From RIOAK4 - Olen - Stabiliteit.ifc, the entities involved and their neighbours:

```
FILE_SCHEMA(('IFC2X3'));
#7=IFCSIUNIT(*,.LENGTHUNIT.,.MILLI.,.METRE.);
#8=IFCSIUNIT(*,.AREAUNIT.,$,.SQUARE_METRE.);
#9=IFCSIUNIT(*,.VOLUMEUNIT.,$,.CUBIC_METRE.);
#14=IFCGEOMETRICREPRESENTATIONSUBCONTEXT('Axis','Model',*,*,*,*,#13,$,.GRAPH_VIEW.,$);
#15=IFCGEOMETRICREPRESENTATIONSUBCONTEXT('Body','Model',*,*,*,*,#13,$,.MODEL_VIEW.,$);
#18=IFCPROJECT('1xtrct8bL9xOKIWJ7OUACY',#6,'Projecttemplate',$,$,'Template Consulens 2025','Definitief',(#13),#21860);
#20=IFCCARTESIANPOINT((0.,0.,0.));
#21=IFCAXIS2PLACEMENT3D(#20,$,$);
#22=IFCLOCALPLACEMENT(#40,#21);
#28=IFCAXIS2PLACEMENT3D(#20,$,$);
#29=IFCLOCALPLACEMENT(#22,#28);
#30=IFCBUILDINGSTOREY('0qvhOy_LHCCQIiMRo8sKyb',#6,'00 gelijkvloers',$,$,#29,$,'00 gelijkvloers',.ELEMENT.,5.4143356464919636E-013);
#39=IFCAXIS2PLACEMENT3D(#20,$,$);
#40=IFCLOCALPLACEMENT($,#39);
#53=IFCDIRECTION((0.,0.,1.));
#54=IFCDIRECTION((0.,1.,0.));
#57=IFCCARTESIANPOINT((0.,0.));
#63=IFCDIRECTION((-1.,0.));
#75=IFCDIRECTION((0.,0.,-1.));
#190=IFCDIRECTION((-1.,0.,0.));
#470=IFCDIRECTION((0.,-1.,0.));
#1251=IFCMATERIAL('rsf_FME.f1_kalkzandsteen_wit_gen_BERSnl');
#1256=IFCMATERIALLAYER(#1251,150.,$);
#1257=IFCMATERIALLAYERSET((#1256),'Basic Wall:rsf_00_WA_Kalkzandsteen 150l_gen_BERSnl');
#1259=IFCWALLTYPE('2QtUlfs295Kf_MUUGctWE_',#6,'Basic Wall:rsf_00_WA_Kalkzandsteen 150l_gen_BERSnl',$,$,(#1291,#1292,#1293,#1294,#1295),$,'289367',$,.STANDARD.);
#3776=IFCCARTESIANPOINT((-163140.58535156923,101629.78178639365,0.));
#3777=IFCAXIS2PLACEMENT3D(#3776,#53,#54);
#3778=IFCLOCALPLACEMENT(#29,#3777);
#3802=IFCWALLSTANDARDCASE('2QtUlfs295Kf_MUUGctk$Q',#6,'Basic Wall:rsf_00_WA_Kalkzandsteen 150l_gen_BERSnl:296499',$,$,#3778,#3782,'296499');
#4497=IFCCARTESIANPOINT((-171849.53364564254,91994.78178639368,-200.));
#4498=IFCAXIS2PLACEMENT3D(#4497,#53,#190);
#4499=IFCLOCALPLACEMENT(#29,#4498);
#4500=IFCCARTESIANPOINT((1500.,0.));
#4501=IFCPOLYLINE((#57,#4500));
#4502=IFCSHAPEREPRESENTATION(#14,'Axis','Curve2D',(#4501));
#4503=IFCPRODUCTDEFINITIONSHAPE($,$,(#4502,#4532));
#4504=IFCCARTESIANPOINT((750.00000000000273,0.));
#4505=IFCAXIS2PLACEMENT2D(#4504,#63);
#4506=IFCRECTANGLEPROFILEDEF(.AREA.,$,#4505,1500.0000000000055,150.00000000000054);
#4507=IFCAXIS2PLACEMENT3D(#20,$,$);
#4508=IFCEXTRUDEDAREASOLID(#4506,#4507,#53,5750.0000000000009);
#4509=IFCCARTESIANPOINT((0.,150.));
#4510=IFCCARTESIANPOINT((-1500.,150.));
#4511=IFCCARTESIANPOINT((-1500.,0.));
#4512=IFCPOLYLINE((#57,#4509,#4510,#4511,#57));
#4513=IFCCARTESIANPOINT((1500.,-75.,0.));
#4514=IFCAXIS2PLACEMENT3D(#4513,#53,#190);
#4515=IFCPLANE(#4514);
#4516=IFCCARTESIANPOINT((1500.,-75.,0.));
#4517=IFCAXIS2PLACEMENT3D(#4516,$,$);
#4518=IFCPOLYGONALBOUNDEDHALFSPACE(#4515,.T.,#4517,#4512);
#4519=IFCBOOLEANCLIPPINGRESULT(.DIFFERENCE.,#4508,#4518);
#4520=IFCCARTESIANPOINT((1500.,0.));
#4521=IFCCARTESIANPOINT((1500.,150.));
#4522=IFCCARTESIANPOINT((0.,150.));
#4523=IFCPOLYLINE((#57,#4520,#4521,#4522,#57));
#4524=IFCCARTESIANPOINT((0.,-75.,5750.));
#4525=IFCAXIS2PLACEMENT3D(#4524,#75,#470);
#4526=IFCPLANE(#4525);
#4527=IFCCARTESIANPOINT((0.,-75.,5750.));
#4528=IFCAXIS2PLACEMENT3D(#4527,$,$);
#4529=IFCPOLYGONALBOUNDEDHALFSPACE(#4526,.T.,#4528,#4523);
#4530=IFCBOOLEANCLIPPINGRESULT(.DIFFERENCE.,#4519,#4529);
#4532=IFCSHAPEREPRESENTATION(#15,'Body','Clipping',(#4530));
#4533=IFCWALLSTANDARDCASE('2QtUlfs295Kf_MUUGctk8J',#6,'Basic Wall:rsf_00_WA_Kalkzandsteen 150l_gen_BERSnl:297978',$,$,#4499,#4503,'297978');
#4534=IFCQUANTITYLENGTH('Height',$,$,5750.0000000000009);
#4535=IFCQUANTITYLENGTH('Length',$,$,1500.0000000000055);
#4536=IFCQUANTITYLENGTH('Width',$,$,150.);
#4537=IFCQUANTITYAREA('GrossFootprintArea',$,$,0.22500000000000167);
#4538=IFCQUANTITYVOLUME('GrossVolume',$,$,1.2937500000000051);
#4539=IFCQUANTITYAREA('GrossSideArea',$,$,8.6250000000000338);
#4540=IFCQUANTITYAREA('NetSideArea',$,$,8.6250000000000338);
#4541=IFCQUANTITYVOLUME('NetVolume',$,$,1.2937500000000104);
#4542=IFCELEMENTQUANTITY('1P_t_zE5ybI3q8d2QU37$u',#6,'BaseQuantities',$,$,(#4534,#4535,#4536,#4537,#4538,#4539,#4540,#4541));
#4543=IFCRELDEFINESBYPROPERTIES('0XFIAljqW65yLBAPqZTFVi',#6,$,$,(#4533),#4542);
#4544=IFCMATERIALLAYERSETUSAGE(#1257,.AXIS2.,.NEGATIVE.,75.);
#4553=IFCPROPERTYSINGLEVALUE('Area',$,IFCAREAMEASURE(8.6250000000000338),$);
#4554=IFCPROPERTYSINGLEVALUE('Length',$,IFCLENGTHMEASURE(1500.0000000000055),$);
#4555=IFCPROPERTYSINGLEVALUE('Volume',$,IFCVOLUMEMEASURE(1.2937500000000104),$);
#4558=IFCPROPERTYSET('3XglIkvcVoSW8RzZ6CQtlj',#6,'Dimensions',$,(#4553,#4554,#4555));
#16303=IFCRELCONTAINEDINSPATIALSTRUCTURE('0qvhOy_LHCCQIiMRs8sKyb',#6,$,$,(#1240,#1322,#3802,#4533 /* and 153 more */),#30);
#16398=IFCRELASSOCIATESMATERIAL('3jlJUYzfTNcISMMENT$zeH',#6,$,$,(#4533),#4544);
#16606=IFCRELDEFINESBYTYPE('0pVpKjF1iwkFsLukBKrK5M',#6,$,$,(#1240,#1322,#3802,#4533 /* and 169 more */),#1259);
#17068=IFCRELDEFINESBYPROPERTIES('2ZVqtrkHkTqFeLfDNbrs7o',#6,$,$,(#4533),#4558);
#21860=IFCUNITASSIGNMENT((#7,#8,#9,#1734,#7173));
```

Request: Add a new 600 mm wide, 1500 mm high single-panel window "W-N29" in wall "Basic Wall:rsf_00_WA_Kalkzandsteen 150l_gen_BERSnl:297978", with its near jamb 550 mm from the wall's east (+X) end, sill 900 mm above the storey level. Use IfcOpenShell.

```python
import numpy as np
import ifcopenshell
import ifcopenshell.api.feature
import ifcopenshell.api.geometry
import ifcopenshell.api.pset
import ifcopenshell.api.root
import ifcopenshell.api.spatial
import ifcopenshell.api.type
import ifcopenshell.geom
import ifcopenshell.util.element
import ifcopenshell.util.placement
import ifcopenshell.util.representation
import ifcopenshell.util.shape
import ifcopenshell.util.unit

model = ifcopenshell.open("RIOAK4 - Olen - Stabiliteit.ifc")
unit_scale = ifcopenshell.util.unit.calculate_unit_scale(model)
area_scale = ifcopenshell.util.unit.calculate_unit_scale(model, "AREAUNIT")
volume_scale = ifcopenshell.util.unit.calculate_unit_scale(model, "VOLUMEUNIT")
settings = ifcopenshell.geom.settings()


def volume(element):
    """Net volume in cubic metres, openings subtracted."""
    shape = ifcopenshell.geom.create_shape(settings, element)
    return ifcopenshell.util.shape.get_volume(shape.geometry)


wall = model.by_id(4533)
storey = ifcopenshell.util.element.get_container(wall, ifc_class="IfcBuildingStorey")
context = ifcopenshell.util.representation.get_context(model, "Model", "Body", "MODEL_VIEW")
before = volume(wall)

width, height, from_end, sill = 0.6, 1.5, 0.55, 0.9  # metres

# The wall runs along its own X axis, and the end named is its -X end.
wall_shape = ifcopenshell.geom.create_shape(settings, wall)
x, y, z = ifcopenshell.util.shape.get_vertices(wall_shape.geometry).T
start = x.min() + from_end
face, thickness = float(y.min()), float(y.max() - y.min())
wall_matrix = ifcopenshell.util.placement.get_local_placement(wall.ObjectPlacement)
level = ifcopenshell.util.placement.get_local_placement(storey.ObjectPlacement)[2, 3]


def in_wall(x, y):
    """Placement at x, y metres in the wall's axes, at sill height."""
    matrix = wall_matrix.copy()
    matrix[:, 3] = wall_matrix @ np.array([x / unit_scale, y / unit_scale, 0.0, 1.0])
    matrix[2, 3] = level + sill / unit_scale
    return matrix


# Opening: a box that overshoots both wall faces by 50 mm.
opening = ifcopenshell.api.root.create_entity(model, ifc_class="IfcOpeningElement")
box = ifcopenshell.api.geometry.add_wall_representation(
    model, context=context, length=width, height=height, thickness=thickness + 0.1
)
ifcopenshell.api.geometry.assign_representation(model, product=opening, representation=box)
ifcopenshell.api.geometry.edit_object_placement(model, product=opening, matrix=in_wall(start, face - 0.05), is_si=False)
ifcopenshell.api.feature.add_feature(model, feature=opening, element=wall)

window = ifcopenshell.api.root.create_entity(model, ifc_class="IfcWindow", name="W-N29")
window.OverallWidth, window.OverallHeight = width / unit_scale, height / unit_scale
body = ifcopenshell.api.geometry.add_window_representation(
    model,
    context=context,
    overall_width=window.OverallWidth,
    overall_height=window.OverallHeight,
    partition_type="SINGLE_PANEL",
)
ifcopenshell.api.geometry.assign_representation(model, product=window, representation=body)
ifcopenshell.api.spatial.assign_container(model, products=[window], relating_structure=storey)
fills = ifcopenshell.api.feature.add_filling(model, opening=opening, element=window)
fills.OwnerHistory = window.OwnerHistory  # required in IFC2X3

# IFC2X3 keeps the operation on the window style.
style = ifcopenshell.api.root.create_entity(model, ifc_class="IfcWindowStyle", name="W-N29")
style.OperationType, style.ConstructionType = "SINGLE_PANEL", "NOTDEFINED"
style.ParameterTakesPrecedence = style.Sizeable = False
ifcopenshell.api.type.assign_type(model, related_objects=[window], relating_type=style)

# Centre the window in the wall's thickness.
ifcopenshell.api.geometry.edit_object_placement(model, product=window, matrix=in_wall(start, face), is_si=False)
window_shape = ifcopenshell.geom.create_shape(settings, window)
depth = ifcopenshell.util.shape.get_vertices(window_shape.geometry)[:, 1]
offset = face + thickness / 2 - (depth.min() + depth.max()) / 2
ifcopenshell.api.geometry.edit_object_placement(model, product=window, matrix=in_wall(start, offset), is_si=False)

after = volume(wall)

# Update the wall's stored quantities.
qto = model.by_id(ifcopenshell.util.element.get_pset(wall, "BaseQuantities", should_inherit=False)["id"])
ifcopenshell.api.pset.edit_qto(model, qto=qto, properties={
    "NetSideArea": after / thickness / area_scale,
    "NetVolume": after / volume_scale,
})
pset = model.by_id(ifcopenshell.util.element.get_pset(wall, "Dimensions", should_inherit=False)["id"])
ifcopenshell.api.pset.edit_pset(model, pset=pset, properties={
    "Area": model.create_entity("IfcAreaMeasure", after / thickness / area_scale),
    "Volume": model.create_entity("IfcVolumeMeasure", after / volume_scale),
})

print(f"wall volume {before:.3f} -> {after:.3f} m3")

model.write("RIOAK4 - Olen - Stabiliteit_v2.ifc")
```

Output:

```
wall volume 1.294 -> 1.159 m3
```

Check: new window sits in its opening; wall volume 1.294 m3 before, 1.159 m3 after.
